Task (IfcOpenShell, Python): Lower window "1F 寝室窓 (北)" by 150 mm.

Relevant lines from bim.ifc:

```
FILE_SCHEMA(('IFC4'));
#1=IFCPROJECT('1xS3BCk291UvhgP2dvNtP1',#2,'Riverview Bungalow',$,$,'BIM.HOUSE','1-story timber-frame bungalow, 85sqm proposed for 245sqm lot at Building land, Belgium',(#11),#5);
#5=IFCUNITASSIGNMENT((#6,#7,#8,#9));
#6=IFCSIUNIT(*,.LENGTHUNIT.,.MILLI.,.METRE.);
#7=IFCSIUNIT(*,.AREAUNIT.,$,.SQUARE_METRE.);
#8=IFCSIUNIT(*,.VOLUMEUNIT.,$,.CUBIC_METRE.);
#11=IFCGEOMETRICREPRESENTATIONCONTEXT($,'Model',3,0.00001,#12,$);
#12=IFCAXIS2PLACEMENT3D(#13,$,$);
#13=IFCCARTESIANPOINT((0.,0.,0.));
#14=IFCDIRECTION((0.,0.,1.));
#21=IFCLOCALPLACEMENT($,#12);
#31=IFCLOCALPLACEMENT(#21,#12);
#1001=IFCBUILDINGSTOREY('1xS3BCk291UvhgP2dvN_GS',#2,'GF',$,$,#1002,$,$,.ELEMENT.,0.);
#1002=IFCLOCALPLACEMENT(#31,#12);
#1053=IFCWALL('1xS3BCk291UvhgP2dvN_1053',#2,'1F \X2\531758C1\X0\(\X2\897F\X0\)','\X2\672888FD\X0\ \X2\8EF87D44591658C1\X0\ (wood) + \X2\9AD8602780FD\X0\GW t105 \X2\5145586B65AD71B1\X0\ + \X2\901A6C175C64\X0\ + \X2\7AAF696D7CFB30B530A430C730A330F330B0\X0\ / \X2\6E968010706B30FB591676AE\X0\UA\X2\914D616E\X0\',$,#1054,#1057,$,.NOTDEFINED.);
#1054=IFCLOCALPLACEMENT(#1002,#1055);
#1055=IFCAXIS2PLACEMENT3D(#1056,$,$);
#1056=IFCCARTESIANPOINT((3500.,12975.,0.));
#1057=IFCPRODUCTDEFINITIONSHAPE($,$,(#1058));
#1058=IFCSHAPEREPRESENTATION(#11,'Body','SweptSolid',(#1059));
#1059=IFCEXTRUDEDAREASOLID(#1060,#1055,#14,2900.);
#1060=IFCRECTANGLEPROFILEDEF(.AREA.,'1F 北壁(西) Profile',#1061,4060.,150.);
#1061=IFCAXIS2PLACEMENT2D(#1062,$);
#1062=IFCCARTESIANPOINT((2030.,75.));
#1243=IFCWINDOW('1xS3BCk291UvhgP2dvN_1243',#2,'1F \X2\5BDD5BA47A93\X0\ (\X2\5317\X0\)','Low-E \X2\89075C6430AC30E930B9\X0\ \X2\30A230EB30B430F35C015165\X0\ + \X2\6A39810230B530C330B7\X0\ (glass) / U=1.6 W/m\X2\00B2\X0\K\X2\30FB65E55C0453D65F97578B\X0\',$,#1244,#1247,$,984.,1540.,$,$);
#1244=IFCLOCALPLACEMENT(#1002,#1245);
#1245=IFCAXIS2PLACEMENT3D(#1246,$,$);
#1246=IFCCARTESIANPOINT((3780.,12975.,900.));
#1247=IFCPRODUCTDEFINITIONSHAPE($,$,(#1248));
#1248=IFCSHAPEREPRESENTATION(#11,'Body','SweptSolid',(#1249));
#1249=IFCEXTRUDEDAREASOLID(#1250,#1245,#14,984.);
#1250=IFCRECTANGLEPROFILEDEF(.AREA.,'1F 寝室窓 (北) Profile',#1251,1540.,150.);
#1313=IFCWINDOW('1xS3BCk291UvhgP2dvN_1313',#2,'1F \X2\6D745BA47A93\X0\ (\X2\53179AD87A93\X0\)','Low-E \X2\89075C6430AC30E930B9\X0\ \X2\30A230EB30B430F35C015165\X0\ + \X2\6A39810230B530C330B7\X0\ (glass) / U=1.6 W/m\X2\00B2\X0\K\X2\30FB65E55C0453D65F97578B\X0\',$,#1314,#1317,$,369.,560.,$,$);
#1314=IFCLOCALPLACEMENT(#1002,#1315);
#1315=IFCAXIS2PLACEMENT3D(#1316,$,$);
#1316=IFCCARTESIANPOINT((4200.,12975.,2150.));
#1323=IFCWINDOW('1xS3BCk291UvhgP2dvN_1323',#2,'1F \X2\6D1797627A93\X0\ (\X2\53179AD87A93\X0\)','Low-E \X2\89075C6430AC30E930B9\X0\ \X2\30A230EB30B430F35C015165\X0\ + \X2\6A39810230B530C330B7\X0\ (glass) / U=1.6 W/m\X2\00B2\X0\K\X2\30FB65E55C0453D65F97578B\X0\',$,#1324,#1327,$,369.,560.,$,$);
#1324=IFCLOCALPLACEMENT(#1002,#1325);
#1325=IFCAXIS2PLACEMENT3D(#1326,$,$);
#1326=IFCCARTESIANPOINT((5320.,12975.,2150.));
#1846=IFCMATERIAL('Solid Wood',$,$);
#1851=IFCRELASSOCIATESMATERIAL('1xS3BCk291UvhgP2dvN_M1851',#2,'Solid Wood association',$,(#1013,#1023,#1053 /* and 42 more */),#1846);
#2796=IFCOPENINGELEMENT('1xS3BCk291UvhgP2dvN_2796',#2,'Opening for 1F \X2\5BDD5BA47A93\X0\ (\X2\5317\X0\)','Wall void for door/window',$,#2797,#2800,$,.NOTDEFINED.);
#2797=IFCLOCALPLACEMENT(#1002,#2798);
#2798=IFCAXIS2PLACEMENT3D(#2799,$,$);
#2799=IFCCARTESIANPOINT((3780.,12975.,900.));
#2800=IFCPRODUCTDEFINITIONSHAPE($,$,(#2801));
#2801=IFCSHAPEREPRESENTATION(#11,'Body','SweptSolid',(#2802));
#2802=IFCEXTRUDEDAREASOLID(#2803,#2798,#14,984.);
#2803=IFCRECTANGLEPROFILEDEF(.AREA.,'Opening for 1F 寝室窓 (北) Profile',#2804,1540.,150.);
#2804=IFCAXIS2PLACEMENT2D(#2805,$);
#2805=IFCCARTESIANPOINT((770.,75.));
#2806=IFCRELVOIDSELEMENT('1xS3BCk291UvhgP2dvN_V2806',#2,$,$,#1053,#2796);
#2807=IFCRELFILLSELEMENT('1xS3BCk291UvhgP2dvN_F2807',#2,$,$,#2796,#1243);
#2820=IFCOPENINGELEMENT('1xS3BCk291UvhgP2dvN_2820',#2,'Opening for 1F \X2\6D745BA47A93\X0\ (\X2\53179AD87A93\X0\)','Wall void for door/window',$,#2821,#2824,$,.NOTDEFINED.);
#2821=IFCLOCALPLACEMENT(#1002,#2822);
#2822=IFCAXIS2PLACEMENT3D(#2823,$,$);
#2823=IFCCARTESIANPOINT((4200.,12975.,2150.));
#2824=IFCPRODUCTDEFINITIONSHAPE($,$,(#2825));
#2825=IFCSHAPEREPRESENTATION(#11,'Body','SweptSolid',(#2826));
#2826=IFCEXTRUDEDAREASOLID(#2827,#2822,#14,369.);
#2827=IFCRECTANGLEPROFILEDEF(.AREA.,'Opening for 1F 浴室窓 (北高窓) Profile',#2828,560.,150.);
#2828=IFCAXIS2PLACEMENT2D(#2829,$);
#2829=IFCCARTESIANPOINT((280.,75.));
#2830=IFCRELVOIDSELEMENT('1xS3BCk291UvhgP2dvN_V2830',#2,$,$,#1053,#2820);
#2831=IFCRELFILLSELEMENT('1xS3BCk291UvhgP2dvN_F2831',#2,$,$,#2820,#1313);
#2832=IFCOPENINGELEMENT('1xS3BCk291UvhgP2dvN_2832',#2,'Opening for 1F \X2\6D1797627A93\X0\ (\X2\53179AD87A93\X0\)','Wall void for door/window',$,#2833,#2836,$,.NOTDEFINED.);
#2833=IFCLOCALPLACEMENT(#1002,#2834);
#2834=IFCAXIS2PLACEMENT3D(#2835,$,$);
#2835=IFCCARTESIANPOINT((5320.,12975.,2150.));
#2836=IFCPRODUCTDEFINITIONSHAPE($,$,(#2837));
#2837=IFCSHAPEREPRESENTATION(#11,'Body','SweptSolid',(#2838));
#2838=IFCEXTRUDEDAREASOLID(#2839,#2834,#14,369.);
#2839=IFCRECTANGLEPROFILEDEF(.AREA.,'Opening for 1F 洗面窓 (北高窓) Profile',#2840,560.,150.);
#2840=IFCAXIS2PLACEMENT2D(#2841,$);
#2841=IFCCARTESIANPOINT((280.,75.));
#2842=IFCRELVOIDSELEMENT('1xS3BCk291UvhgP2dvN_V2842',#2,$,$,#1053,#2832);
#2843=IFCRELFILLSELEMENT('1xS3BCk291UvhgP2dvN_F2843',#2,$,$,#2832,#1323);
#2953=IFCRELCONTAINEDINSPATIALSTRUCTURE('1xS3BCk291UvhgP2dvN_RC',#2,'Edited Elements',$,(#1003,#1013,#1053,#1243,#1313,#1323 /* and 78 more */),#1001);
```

```python
import numpy as np
import ifcopenshell
import ifcopenshell.api.geometry
import ifcopenshell.util.placement
import ifcopenshell.util.unit

model = ifcopenshell.open("bim.ifc")
unit_scale = ifcopenshell.util.unit.calculate_unit_scale(model)

window = model.by_guid("1xS3BCk291UvhgP2dvN_1243")
opening = window.FillsVoids[0].RelatingOpeningElement
dz = -150.0

shift = np.array([0.0, 0.0, dz])
# The window is not placed relative to its opening, so move both.
for product in (opening, window):
    matrix = ifcopenshell.util.placement.get_local_placement(product.ObjectPlacement)
    matrix[:3, 3] += shift
    ifcopenshell.api.geometry.edit_object_placement(model, product=product, matrix=matrix, is_si=False)

print(f"moved by {dz * unit_scale:+.3f} m")

model.write("bim_updated.ifc")
```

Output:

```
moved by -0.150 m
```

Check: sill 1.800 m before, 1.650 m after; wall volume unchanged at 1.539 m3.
